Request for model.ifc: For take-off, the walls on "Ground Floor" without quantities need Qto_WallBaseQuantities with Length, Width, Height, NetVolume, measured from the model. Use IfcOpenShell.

First a look at what the model holds.

```python
import ifcopenshell
import ifcopenshell.util.element
import ifcopenshell.util.unit

model = ifcopenshell.open("model.ifc")
print(model.schema)
for unit_type in ("LENGTHUNIT", "AREAUNIT", "VOLUMEUNIT"):
    print(unit_type, ifcopenshell.util.unit.calculate_unit_scale(model, unit_type))
storey = next(s for s in model.by_type("IfcBuildingStorey") if s.Name == "Ground Floor")
walls = [e for e in ifcopenshell.util.element.get_decomposition(storey) if e.is_a("IfcWall")]
for e in sorted(walls, key=lambda e: e.id()):
    print(e.id(), e.is_a(), e.Name, list(ifcopenshell.util.element.get_psets(e, qtos_only=True)), sep=" | ")
```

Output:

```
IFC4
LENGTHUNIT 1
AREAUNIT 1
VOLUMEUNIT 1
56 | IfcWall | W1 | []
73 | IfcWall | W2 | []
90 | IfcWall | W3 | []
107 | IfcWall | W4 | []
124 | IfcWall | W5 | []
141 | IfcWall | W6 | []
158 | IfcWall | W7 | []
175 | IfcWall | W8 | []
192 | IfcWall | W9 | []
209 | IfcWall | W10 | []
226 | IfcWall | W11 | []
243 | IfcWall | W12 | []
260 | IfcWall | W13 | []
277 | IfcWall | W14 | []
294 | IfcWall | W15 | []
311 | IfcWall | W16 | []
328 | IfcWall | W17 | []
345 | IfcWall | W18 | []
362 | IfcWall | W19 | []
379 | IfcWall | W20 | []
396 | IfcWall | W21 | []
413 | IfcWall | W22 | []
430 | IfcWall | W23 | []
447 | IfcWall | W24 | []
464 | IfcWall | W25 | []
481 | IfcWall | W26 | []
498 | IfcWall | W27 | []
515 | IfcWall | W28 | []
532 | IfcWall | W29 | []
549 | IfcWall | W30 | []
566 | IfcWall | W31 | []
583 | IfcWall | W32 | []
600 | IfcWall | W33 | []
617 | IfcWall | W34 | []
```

```python
import ifcopenshell
import ifcopenshell.api.pset
import ifcopenshell.geom
import ifcopenshell.util.element
import ifcopenshell.util.shape
import ifcopenshell.util.unit

model = ifcopenshell.open("model.ifc")
unit_scale = ifcopenshell.util.unit.calculate_unit_scale(model)
volume_scale = ifcopenshell.util.unit.calculate_unit_scale(model, "VOLUMEUNIT")
settings = ifcopenshell.geom.settings()

storey = next(s for s in model.by_type("IfcBuildingStorey") if s.Name == "Ground Floor")
walls = [e for e in ifcopenshell.util.element.get_decomposition(storey) if e.is_a("IfcWall")]

for e in sorted(walls, key=lambda e: e.id()):
    if ifcopenshell.util.element.get_psets(e, qtos_only=True, should_inherit=False):
        continue
    # Geometry comes back in metres, in the element's own axes.
    shape = ifcopenshell.geom.create_shape(settings, e)
    values = {
        "Length": ifcopenshell.util.shape.get_x(shape.geometry) / unit_scale,
        "Width": ifcopenshell.util.shape.get_y(shape.geometry) / unit_scale,
        "Height": ifcopenshell.util.shape.get_z(shape.geometry) / unit_scale,
        "NetVolume": ifcopenshell.util.shape.get_volume(shape.geometry) / volume_scale,
    }
    qto = ifcopenshell.api.pset.add_qto(model, product=e, name="Qto_WallBaseQuantities")
    ifcopenshell.api.pset.edit_qto(model, qto=qto, properties=values)
    print(e.id(), {k: round(v, 3) for k, v in values.items()})

model.write("model_edited.ifc")
```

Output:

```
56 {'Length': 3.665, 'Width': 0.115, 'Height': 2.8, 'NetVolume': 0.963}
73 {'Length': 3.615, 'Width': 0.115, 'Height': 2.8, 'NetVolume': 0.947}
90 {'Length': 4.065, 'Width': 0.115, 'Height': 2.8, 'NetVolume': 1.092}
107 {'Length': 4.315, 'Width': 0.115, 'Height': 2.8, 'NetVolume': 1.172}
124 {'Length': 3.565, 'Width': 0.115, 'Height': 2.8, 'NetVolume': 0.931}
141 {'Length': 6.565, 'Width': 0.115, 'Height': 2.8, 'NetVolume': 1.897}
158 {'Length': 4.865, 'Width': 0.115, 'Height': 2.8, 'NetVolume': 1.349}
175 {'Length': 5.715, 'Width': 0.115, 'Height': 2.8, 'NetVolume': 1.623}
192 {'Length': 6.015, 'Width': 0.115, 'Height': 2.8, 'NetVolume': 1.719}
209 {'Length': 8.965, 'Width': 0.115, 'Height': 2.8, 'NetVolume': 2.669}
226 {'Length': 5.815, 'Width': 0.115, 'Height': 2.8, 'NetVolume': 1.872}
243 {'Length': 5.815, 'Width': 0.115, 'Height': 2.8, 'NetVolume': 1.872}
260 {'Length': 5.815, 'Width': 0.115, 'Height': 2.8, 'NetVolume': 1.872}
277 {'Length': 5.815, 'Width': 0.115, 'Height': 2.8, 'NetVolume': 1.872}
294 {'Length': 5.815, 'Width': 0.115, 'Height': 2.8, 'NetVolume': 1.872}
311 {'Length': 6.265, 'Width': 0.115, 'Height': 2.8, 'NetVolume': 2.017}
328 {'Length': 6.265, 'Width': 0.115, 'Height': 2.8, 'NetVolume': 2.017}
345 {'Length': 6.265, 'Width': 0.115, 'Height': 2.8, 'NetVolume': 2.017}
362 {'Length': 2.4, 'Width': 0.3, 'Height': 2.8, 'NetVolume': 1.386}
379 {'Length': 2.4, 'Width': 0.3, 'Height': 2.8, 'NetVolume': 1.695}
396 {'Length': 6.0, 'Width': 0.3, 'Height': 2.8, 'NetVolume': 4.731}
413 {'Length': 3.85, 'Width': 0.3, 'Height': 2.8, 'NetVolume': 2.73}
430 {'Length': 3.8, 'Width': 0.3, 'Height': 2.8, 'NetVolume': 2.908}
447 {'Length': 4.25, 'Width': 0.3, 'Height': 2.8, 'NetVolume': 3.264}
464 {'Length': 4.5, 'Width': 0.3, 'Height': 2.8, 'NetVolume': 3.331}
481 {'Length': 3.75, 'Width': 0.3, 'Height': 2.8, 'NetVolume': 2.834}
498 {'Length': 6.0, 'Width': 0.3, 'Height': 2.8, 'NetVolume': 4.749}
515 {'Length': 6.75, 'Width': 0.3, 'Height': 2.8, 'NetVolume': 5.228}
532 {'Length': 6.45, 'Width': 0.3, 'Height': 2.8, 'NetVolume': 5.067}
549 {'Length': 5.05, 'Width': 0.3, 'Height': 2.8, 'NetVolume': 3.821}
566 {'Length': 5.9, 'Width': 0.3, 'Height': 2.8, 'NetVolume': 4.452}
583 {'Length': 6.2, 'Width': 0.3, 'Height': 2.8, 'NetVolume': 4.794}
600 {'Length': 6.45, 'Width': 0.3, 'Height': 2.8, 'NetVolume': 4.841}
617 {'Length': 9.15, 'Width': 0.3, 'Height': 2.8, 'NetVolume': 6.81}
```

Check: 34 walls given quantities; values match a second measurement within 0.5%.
